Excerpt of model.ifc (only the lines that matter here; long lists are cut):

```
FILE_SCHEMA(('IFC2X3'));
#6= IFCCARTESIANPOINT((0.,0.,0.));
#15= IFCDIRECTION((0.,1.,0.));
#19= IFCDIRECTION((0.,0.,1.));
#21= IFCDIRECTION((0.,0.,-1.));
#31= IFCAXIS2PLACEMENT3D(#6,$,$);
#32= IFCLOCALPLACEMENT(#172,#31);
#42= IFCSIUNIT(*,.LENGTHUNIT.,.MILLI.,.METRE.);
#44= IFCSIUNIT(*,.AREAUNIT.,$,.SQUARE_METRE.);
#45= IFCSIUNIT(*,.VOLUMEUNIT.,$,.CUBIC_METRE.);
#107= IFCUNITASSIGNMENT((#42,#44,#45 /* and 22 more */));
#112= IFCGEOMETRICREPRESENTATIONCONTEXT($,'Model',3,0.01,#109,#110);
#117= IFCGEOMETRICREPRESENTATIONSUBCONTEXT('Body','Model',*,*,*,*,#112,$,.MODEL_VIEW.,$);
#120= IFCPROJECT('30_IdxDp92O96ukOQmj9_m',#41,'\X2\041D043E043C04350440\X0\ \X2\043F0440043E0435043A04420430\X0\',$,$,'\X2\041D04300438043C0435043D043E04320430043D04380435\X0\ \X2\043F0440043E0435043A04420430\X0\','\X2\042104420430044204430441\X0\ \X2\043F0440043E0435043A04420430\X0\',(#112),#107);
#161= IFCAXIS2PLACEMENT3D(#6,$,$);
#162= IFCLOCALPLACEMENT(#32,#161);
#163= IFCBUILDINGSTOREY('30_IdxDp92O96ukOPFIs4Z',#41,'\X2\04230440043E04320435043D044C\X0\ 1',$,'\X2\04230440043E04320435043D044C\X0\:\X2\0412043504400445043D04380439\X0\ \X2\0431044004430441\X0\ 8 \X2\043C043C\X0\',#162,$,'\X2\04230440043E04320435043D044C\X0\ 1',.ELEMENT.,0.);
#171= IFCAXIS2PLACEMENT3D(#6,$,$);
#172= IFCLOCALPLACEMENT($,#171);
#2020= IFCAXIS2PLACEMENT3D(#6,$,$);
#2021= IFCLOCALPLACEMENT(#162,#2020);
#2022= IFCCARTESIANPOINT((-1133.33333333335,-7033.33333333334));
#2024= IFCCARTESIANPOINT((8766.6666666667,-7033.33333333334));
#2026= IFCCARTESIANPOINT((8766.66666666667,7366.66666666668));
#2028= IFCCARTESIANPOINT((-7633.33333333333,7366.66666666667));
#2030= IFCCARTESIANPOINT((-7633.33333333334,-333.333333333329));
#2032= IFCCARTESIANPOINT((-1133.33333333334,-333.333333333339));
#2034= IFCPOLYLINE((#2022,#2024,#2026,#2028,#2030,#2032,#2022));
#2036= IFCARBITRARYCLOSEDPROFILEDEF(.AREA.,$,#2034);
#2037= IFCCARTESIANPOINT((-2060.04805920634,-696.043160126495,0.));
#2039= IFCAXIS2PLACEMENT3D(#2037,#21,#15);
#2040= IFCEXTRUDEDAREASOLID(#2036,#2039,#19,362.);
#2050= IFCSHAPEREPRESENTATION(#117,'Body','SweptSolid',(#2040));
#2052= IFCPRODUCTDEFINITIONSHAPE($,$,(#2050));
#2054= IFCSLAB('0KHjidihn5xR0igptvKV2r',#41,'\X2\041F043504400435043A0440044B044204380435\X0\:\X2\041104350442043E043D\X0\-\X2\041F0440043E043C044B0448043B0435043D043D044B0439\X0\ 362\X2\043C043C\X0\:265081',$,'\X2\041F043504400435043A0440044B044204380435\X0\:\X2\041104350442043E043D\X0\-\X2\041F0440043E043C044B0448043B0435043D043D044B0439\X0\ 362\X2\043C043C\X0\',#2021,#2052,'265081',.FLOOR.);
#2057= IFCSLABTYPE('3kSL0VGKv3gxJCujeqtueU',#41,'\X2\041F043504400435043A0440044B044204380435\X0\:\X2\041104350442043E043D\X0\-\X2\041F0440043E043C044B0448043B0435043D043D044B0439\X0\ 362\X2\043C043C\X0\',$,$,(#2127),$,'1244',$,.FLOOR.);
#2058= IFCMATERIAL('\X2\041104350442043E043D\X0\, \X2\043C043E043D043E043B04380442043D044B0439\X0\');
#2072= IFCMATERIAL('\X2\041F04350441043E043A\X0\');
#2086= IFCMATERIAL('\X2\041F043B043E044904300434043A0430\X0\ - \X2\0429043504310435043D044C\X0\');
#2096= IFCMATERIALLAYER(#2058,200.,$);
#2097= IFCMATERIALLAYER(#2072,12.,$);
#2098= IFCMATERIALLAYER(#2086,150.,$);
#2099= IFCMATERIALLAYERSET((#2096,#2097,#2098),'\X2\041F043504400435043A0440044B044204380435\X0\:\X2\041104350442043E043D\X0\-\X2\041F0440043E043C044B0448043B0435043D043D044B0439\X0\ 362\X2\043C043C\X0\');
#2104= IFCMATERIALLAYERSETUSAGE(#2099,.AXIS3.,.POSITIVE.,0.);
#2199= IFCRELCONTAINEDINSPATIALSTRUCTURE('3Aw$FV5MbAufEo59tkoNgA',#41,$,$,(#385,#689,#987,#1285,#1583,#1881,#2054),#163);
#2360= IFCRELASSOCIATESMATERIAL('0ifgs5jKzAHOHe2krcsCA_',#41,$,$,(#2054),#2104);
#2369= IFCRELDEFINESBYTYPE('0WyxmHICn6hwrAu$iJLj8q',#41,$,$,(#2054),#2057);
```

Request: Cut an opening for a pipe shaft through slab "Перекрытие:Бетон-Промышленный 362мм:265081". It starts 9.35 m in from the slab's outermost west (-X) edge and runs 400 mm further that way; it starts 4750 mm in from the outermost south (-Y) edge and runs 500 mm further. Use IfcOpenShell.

```python
import numpy as np
import ifcopenshell
import ifcopenshell.api.feature
import ifcopenshell.api.geometry
import ifcopenshell.api.root
import ifcopenshell.geom
import ifcopenshell.util.placement
import ifcopenshell.util.representation
import ifcopenshell.util.shape
import ifcopenshell.util.unit

model = ifcopenshell.open("model.ifc")
unit_scale = ifcopenshell.util.unit.calculate_unit_scale(model)
settings = ifcopenshell.geom.settings()


def volume(element):
    """Net volume in cubic metres, openings subtracted."""
    shape = ifcopenshell.geom.create_shape(settings, element)
    return ifcopenshell.util.shape.get_volume(shape.geometry)


slab = model.by_id(2054)
before = volume(slab)

# Extent in the slab's own axes, in metres. The edges named are its -X and -Y sides.
slab_shape = ifcopenshell.geom.create_shape(settings, slab)
vertices = ifcopenshell.util.shape.get_vertices(slab_shape.geometry)
x_min, y_min, bottom = vertices.min(axis=0)
top = vertices[:, 2].max()

opening = ifcopenshell.api.root.create_entity(model, ifc_class="IfcOpeningElement", name="Pipe shaft opening")
context = ifcopenshell.util.representation.get_context(model, "Model", "Body", "MODEL_VIEW")
width, depth = 0.4, 0.5
outline = [(0.0, 0.0), (width, 0.0), (width, depth), (0.0, depth), (0.0, 0.0)]
# Overshoot both faces by 50 mm so the cut is clean.
shape = ifcopenshell.api.geometry.add_slab_representation(
    model, context=context, depth=top - bottom + 0.1, polyline=outline
)
ifcopenshell.api.geometry.assign_representation(model, product=opening, representation=shape)

matrix = ifcopenshell.util.placement.get_local_placement(slab.ObjectPlacement)
matrix[:, 3] = matrix @ np.append(np.array([x_min + 9.35, y_min + 4.75, bottom - 0.05]) / unit_scale, 1.0)
ifcopenshell.api.geometry.edit_object_placement(model, product=opening, matrix=matrix, is_si=False)
ifcopenshell.api.feature.add_feature(model, feature=opening, element=slab)

after = volume(slab)

print(f"slab volume {before:.3f} -> {after:.3f} m3")

model.write("model_edited.ifc")
```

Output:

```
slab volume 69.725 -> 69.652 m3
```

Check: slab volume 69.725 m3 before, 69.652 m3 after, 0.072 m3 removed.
